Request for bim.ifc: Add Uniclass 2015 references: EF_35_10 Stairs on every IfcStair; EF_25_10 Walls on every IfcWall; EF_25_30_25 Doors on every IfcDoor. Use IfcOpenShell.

First a look at what the model holds.

```python
import ifcopenshell

model = ifcopenshell.open("bim.ifc")
print(model.schema)
print("classifications:", [c.Name for c in model.by_type("IfcClassification")])
for ifc_class in ("IfcDoor", "IfcRoof", "IfcStair", "IfcWall", "IfcWindow"):
    print(ifc_class, len(model.by_type(ifc_class)))
```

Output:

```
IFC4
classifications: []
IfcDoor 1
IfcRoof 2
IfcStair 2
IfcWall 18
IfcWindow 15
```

```python
import ifcopenshell
import ifcopenshell.api.classification

model = ifcopenshell.open("bim.ifc")

system = ifcopenshell.api.classification.add_classification(model, classification="Uniclass 2015")

codes = {
    "IfcStair": ("EF_35_10", "Stairs"),
    "IfcWall": ("EF_25_10", "Walls"),
    "IfcDoor": ("EF_25_30_25", "Doors"),
}
for ifc_class, (code, name) in codes.items():
    products = model.by_type(ifc_class)
    ifcopenshell.api.classification.add_reference(
        model, products=products, classification=system, identification=code, name=name
    )
    print(code, len(products))

model.write("bim-out.ifc")
```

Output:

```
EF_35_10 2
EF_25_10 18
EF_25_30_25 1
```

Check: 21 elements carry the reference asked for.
